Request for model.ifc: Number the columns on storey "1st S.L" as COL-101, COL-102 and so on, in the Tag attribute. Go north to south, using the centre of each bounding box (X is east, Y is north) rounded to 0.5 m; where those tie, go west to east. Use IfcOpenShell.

First a look at what the model holds.

```python
import ifcopenshell
import ifcopenshell.util.element
import ifcopenshell.util.placement

model = ifcopenshell.open("model.ifc")
print(model.schema)
storey = next(s for s in model.by_type("IfcBuildingStorey") if s.Name == "1st S.L")
columns = [e for e in ifcopenshell.util.element.get_decomposition(storey) if e.is_a("IfcColumn")]
for e in sorted(columns, key=lambda e: e.id()):
    origin = ifcopenshell.util.placement.get_local_placement(e.ObjectPlacement)[:3, 3]
    print(e.id(), e.Tag, e.Name, origin.round(2) + 0.0, sep=" | ")
```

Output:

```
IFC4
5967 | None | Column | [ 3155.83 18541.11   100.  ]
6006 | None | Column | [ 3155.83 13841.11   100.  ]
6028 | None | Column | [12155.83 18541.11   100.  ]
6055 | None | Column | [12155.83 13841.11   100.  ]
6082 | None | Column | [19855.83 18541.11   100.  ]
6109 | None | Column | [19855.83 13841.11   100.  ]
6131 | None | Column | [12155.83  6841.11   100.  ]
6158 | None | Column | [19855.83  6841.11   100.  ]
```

```python
import ifcopenshell
import ifcopenshell.geom
import ifcopenshell.util.element
import ifcopenshell.util.shape

model = ifcopenshell.open("model.ifc")
settings = ifcopenshell.geom.settings()
settings.set("use-world-coords", True)


def centre(element):
    shape = ifcopenshell.geom.create_shape(settings, element)
    return ifcopenshell.util.shape.get_bbox_centroid(shape.geometry)


storey = next(s for s in model.by_type("IfcBuildingStorey") if s.Name == "1st S.L")
columns = [e for e in ifcopenshell.util.element.get_decomposition(storey) if e.is_a("IfcColumn")]

# Insertion points can sit at a corner or the storey origin, so sort by the geometry (in metres).
centres = {e: centre(e) for e in columns}
columns.sort(key=lambda e: (-round(centres[e][1] / 0.5), centres[e][0]))

for i, e in enumerate(columns, start=1):
    number = f"COL-1{i:02d}"
    e.Tag = number
    print(e.id(), number)

model.write("model_updated.ifc")
```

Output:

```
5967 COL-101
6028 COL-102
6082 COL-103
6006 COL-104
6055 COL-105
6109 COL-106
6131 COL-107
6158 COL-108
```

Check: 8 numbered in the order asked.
